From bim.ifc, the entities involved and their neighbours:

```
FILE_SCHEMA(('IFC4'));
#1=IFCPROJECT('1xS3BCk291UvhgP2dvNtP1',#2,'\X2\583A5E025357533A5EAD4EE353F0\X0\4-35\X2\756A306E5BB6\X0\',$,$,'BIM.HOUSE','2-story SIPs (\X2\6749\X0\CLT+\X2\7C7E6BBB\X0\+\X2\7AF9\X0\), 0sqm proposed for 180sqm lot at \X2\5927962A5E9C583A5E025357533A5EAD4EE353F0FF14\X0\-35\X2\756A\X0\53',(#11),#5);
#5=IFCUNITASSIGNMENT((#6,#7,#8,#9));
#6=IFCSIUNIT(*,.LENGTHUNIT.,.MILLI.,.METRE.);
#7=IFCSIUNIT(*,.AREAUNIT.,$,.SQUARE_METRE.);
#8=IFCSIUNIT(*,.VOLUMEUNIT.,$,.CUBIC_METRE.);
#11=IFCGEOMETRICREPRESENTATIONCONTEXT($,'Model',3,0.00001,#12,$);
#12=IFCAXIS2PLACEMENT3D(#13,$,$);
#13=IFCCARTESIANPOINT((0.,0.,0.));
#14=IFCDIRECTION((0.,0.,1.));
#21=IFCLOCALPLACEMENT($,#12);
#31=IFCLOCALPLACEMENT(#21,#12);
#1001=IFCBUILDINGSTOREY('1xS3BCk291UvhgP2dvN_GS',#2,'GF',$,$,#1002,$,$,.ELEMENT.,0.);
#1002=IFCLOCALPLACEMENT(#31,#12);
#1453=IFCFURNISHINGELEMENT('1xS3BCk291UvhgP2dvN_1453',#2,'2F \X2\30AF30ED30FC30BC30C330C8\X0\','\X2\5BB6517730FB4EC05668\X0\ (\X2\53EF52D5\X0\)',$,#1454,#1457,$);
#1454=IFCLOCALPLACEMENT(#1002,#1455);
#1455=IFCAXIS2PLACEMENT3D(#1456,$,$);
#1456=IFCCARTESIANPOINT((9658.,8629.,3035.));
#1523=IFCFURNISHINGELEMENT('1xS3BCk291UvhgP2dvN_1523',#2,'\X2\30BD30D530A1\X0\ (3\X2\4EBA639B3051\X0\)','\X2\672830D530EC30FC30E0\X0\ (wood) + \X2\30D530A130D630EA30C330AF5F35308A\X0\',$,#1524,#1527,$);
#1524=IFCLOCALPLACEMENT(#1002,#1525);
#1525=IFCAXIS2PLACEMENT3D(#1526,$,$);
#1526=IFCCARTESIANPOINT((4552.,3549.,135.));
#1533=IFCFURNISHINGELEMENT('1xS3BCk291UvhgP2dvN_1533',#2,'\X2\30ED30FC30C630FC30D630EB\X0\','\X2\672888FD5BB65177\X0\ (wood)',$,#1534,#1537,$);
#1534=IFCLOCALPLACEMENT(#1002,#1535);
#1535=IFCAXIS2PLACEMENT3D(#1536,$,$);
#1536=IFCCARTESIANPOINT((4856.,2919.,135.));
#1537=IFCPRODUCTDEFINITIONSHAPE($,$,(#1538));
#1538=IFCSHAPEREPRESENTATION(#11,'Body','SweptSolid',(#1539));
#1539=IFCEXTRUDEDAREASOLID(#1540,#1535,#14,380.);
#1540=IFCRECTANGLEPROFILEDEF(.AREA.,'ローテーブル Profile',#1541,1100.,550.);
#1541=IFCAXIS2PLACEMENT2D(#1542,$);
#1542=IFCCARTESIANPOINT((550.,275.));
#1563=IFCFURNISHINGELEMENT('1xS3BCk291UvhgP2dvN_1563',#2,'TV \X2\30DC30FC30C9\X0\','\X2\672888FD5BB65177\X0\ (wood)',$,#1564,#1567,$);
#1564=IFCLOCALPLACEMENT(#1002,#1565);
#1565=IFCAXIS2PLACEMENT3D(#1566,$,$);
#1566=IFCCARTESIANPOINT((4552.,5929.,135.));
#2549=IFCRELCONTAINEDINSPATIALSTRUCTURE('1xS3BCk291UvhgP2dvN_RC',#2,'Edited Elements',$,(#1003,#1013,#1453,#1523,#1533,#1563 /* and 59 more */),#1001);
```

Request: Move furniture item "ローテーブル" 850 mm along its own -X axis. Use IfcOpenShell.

```python
import ifcopenshell
import ifcopenshell.api.geometry
import ifcopenshell.util.placement
import ifcopenshell.util.unit

model = ifcopenshell.open("bim.ifc")
unit_scale = ifcopenshell.util.unit.calculate_unit_scale(model)

item = model.by_guid("1xS3BCk291UvhgP2dvN_1533")
matrix = ifcopenshell.util.placement.get_local_placement(item.ObjectPlacement)
matrix[:3, 3] -= matrix[:3, 0] * 0.85 / unit_scale
ifcopenshell.api.geometry.edit_object_placement(model, product=item, matrix=matrix, is_si=False)

print(ifcopenshell.util.placement.get_local_placement(item.ObjectPlacement).round(3) + 0.0)

model.write("bim_updated.ifc")
```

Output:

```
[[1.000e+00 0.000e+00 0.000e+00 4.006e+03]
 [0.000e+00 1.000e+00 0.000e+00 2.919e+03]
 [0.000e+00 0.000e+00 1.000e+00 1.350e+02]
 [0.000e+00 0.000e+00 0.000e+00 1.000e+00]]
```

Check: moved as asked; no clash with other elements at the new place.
